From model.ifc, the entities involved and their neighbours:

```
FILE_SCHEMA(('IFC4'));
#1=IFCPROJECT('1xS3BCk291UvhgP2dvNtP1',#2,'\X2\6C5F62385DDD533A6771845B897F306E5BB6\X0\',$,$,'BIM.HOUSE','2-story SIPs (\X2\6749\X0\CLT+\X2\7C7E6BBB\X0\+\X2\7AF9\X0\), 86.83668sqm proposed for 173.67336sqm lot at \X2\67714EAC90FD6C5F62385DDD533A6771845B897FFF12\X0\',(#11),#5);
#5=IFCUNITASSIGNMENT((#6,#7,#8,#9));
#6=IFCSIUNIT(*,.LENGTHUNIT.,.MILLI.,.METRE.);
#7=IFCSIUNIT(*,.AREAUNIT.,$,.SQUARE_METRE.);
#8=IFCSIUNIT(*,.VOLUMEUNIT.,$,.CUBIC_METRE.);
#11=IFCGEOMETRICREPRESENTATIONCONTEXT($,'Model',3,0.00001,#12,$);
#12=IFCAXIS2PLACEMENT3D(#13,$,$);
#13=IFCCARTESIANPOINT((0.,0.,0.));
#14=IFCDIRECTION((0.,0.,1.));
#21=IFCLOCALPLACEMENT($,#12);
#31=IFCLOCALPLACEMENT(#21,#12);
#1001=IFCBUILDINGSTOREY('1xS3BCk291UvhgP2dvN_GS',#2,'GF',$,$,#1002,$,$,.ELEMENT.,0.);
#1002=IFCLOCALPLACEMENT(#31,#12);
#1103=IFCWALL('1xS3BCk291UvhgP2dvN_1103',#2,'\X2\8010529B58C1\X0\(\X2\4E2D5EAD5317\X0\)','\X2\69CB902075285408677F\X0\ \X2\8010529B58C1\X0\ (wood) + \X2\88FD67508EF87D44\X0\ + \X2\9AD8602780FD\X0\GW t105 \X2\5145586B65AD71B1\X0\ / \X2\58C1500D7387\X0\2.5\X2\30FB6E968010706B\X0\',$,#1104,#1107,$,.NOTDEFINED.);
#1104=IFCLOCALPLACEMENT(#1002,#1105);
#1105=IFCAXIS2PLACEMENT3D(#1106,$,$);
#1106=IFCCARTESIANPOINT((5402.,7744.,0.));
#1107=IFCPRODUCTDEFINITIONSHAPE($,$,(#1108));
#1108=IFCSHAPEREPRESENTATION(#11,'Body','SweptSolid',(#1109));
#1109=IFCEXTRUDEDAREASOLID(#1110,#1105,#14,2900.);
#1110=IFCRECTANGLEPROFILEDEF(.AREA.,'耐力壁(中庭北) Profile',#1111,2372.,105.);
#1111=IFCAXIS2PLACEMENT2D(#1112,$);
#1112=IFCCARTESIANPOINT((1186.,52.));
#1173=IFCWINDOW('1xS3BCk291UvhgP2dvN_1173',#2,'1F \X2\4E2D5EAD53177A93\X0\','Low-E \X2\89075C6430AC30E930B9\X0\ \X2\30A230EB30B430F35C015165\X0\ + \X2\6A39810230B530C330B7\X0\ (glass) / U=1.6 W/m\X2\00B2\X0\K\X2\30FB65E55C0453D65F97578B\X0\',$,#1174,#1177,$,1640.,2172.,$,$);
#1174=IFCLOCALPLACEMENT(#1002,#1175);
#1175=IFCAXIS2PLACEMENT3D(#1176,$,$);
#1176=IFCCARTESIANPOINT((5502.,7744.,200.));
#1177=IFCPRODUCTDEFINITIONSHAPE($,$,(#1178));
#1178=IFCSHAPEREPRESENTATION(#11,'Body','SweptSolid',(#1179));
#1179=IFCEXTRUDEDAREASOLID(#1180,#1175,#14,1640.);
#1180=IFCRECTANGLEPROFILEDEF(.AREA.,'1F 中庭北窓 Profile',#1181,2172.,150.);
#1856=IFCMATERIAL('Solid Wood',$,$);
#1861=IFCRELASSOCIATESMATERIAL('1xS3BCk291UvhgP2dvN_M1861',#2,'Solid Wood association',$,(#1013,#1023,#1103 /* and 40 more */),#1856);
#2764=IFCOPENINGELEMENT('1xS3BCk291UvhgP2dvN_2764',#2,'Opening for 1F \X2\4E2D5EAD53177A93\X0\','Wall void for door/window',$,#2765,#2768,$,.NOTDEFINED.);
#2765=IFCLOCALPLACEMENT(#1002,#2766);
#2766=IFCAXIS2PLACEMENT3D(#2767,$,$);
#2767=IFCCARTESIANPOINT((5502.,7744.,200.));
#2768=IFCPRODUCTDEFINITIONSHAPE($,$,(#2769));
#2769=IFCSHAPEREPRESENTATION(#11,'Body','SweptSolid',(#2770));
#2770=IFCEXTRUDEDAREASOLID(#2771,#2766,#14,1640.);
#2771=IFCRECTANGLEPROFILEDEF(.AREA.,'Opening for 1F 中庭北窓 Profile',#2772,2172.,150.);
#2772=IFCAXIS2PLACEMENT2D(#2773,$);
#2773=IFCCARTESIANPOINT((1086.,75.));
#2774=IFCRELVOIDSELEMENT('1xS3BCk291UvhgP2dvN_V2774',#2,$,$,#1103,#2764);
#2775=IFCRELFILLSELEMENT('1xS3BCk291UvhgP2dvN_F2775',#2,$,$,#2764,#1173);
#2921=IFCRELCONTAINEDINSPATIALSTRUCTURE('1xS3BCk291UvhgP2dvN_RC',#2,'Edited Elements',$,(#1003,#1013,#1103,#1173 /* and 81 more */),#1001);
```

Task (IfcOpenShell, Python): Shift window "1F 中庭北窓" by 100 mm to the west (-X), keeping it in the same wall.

```python
import ifcopenshell
import ifcopenshell.api.geometry
import ifcopenshell.util.placement
import ifcopenshell.util.unit

model = ifcopenshell.open("model.ifc")
unit_scale = ifcopenshell.util.unit.calculate_unit_scale(model)

window = model.by_guid("1xS3BCk291UvhgP2dvN_1173")
opening = window.FillsVoids[0].RelatingOpeningElement
wall = opening.VoidsElements[0].RelatingBuildingElement

wall_matrix = ifcopenshell.util.placement.get_local_placement(wall.ObjectPlacement)
shift = wall_matrix[:3, 0] * -0.1 / unit_scale
before = ifcopenshell.util.placement.get_local_placement(window.ObjectPlacement)[:3, 3].copy()

# The window is not placed relative to its opening, so move both.
for product in (opening, window):
    matrix = ifcopenshell.util.placement.get_local_placement(product.ObjectPlacement)
    matrix[:3, 3] += shift
    ifcopenshell.api.geometry.edit_object_placement(model, product=product, matrix=matrix, is_si=False)

after = ifcopenshell.util.placement.get_local_placement(window.ObjectPlacement)[:3, 3]
print("window moved by", (after - before).round(3) + 0.0)

model.write("model_edited.ifc")
```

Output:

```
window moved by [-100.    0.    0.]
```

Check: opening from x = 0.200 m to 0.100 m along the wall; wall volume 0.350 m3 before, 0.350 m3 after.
